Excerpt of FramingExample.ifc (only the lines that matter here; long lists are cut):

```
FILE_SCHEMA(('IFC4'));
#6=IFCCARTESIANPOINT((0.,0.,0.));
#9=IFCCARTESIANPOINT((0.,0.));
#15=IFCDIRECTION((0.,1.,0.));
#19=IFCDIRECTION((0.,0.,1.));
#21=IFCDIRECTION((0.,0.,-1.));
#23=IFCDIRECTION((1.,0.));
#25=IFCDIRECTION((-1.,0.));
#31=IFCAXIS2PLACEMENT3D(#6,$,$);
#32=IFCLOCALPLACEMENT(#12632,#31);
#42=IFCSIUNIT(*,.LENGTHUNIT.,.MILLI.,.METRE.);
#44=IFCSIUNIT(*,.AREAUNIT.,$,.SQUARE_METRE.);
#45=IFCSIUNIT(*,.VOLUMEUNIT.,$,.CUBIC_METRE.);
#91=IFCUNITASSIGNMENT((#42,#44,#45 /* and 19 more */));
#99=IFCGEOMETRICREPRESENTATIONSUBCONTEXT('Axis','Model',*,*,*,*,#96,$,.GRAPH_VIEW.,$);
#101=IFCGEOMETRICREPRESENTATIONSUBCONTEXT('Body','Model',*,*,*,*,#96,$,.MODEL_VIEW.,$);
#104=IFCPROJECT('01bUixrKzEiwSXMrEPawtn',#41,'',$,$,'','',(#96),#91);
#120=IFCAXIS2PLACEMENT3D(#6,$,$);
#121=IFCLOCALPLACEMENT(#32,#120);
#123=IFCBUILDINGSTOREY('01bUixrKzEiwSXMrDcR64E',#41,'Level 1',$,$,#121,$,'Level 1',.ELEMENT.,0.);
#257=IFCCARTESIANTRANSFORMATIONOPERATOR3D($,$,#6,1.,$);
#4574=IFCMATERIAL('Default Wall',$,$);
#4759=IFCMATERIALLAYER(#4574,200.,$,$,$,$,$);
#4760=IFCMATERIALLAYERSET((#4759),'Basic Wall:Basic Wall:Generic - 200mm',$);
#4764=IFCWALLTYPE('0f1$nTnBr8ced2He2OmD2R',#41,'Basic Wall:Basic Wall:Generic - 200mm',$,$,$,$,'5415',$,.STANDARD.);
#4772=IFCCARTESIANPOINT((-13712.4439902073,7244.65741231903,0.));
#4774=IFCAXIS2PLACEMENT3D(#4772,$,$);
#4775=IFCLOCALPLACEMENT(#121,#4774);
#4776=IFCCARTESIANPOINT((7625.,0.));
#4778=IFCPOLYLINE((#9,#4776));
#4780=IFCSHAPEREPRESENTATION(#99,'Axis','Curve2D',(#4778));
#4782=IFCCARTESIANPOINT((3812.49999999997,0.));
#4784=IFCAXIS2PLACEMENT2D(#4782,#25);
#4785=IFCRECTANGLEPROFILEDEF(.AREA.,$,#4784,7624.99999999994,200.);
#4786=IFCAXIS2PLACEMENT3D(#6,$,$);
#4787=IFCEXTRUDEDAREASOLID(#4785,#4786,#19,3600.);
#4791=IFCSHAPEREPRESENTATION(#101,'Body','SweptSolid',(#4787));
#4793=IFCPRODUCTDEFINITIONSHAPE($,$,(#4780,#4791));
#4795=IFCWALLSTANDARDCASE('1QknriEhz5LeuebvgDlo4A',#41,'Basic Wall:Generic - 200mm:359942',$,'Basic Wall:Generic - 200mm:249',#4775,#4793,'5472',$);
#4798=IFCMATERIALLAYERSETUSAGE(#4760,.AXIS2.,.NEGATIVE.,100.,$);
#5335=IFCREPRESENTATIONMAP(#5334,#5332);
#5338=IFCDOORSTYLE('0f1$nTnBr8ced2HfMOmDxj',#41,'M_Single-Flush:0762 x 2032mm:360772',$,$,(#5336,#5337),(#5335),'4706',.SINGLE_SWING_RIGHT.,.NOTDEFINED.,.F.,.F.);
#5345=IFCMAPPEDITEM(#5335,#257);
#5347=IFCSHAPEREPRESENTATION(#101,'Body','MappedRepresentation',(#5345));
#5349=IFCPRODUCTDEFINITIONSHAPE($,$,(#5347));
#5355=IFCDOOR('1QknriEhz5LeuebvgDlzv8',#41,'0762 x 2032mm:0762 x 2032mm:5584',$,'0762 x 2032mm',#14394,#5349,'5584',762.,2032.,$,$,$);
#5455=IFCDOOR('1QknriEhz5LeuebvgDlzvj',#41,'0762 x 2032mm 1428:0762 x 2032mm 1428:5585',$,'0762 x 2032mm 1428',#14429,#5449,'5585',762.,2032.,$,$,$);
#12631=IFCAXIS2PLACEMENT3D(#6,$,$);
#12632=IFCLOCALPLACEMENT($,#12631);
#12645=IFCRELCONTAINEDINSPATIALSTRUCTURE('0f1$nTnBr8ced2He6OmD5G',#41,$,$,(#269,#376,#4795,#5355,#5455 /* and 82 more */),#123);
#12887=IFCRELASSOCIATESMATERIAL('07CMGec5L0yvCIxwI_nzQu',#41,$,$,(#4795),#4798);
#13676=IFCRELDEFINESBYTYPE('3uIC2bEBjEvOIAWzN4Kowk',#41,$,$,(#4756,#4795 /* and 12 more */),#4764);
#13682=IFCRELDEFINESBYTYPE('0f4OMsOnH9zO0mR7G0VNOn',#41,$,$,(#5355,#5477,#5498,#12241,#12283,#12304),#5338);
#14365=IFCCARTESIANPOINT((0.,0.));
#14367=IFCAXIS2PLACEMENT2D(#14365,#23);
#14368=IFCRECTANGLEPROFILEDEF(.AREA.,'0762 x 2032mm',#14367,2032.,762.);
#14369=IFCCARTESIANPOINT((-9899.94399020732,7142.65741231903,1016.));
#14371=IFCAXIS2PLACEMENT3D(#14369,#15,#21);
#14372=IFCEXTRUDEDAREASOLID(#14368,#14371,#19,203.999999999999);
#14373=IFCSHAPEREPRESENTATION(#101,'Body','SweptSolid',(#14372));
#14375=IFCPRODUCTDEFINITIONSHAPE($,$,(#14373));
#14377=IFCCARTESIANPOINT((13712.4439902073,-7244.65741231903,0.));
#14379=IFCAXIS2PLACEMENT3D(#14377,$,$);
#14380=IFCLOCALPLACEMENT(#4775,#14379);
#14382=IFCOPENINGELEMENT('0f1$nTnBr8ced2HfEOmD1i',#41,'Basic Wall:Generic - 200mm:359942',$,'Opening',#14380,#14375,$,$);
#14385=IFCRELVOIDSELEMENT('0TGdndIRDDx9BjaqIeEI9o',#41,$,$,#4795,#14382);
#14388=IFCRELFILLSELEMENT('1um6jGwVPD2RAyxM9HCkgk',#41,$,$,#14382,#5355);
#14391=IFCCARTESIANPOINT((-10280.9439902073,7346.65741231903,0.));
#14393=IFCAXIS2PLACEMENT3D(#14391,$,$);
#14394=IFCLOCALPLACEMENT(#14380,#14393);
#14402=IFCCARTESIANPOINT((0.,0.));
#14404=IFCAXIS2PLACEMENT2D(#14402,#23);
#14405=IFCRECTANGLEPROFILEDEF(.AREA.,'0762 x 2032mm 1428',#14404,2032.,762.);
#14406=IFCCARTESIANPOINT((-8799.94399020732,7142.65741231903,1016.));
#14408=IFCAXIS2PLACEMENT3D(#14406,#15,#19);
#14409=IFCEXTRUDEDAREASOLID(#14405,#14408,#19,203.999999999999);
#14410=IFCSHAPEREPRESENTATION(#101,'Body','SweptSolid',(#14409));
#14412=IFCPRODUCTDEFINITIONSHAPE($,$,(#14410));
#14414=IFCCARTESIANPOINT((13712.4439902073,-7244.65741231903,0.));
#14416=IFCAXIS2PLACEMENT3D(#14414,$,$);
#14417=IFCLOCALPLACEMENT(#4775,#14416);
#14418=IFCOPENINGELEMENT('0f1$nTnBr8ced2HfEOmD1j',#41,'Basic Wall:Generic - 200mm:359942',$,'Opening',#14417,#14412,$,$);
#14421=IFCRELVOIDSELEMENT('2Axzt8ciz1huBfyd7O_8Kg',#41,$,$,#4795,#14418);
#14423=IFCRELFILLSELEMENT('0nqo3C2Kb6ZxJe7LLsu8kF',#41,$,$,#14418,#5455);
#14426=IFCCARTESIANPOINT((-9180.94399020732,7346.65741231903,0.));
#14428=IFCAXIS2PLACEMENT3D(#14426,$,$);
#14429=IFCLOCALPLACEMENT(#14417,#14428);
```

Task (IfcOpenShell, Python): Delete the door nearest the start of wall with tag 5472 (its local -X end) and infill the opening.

```python
import ifcopenshell
import ifcopenshell.api.feature
import ifcopenshell.api.root
import ifcopenshell.geom
import ifcopenshell.util.shape

model = ifcopenshell.open("FramingExample.ifc")
settings = ifcopenshell.geom.settings()


def volume(element):
    """Net volume in cubic metres, openings subtracted."""
    shape = ifcopenshell.geom.create_shape(settings, element)
    return ifcopenshell.util.shape.get_volume(shape.geometry)


door = model.by_guid("1QknriEhz5LeuebvgDlzv8")
opening = door.FillsVoids[0].RelatingOpeningElement
wall = opening.VoidsElements[0].RelatingBuildingElement
before = volume(wall)

ifcopenshell.api.root.remove_product(model, product=door)
ifcopenshell.api.feature.remove_feature(model, feature=opening)

after = volume(wall)

print(f"wall volume {before:.3f} -> {after:.3f} m3")

model.write("FramingExample_updated.ifc")
```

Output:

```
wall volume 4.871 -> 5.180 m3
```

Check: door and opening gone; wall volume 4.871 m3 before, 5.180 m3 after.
